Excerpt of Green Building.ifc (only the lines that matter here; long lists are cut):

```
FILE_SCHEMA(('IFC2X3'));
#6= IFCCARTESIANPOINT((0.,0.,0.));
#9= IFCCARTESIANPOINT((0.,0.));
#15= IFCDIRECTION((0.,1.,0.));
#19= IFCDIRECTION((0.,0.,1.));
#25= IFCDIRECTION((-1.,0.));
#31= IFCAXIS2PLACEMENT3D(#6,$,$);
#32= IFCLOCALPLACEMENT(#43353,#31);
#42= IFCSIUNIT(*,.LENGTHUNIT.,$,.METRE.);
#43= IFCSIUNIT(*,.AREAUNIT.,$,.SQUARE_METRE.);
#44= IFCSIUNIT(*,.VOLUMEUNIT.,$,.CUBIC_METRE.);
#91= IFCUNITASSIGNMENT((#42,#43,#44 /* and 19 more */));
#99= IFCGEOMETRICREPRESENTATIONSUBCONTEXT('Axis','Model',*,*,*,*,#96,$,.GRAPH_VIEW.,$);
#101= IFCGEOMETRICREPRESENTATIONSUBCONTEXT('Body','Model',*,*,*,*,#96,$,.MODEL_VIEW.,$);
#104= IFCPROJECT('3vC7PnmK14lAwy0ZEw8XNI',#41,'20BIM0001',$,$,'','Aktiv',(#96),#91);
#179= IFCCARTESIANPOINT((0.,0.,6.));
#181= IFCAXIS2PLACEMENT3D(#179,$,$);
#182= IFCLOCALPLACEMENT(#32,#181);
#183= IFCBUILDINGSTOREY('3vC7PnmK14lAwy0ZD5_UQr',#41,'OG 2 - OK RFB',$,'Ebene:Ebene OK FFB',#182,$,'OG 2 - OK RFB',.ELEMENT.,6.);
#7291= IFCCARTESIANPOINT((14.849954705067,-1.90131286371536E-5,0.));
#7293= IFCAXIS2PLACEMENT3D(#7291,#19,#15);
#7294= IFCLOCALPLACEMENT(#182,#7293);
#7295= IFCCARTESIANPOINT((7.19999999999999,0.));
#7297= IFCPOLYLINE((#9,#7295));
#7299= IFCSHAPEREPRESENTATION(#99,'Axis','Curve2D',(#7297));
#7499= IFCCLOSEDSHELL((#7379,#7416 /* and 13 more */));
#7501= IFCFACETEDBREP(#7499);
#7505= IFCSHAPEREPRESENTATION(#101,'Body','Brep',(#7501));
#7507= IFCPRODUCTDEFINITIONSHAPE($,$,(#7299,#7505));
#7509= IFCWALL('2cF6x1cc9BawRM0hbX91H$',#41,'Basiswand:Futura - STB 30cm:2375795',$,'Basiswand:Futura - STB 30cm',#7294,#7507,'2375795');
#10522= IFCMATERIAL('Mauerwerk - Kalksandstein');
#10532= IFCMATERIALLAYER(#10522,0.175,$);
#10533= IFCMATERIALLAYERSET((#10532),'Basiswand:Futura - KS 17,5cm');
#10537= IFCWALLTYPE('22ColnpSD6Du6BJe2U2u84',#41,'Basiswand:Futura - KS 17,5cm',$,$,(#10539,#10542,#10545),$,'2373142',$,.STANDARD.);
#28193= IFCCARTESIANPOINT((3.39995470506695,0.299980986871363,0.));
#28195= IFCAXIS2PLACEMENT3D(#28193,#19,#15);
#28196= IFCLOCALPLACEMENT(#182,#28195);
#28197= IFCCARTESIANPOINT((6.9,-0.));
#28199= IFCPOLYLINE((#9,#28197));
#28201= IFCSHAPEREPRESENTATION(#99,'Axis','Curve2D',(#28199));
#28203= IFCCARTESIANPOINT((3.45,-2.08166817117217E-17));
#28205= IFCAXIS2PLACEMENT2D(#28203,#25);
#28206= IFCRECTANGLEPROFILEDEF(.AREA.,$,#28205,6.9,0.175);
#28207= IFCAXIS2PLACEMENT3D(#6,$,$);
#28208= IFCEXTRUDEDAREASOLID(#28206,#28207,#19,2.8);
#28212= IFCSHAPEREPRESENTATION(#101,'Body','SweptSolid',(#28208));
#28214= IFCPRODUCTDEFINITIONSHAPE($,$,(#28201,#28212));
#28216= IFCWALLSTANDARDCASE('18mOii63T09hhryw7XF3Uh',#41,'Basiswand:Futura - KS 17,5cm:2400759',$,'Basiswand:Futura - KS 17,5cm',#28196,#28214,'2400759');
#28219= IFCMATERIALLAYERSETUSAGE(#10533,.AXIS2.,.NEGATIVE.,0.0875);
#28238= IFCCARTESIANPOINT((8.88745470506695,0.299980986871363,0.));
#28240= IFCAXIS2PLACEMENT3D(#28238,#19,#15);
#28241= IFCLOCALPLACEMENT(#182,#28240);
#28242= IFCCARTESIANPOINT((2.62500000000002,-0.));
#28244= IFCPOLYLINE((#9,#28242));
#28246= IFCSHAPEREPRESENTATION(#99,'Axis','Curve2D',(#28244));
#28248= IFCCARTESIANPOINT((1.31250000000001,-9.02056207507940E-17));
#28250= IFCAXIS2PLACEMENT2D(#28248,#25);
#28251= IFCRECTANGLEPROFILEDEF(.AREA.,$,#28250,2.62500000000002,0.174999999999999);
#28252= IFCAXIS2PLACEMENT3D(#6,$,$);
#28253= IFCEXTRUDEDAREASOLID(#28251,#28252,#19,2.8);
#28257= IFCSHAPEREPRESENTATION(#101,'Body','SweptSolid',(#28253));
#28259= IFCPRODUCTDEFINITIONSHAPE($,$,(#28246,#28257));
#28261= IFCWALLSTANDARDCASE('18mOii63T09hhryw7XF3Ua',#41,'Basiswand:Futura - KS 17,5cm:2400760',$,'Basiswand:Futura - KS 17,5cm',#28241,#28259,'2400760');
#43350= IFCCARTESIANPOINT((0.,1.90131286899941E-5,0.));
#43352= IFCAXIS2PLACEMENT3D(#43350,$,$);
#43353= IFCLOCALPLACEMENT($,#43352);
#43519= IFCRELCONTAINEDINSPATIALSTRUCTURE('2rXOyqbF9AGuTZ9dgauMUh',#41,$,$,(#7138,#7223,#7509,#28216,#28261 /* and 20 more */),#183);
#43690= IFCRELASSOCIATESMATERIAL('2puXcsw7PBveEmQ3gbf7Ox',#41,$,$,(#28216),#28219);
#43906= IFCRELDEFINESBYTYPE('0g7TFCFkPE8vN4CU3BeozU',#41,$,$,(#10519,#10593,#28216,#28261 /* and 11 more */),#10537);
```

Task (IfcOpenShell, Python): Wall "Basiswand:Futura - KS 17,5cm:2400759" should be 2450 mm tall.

```python
import ifcopenshell
import ifcopenshell.geom
import ifcopenshell.util.representation
import ifcopenshell.util.shape
import ifcopenshell.util.unit

model = ifcopenshell.open("Green Building.ifc")
unit_scale = ifcopenshell.util.unit.calculate_unit_scale(model)
settings = ifcopenshell.geom.settings()


def volume(element):
    """Net volume in cubic metres, openings subtracted."""
    shape = ifcopenshell.geom.create_shape(settings, element)
    return ifcopenshell.util.shape.get_volume(shape.geometry)


wall = model.by_id(28216)
before = volume(wall)

body = ifcopenshell.util.representation.get_representation(wall, "Model", "Body")
solid = body.Items[0]
old_height = solid.Depth
solid.Depth = 2.45 / unit_scale
after = volume(wall)

print(f"height {old_height:g} -> {solid.Depth:g}, volume {before:.3f} -> {after:.3f} m3")

model.write("Green Building-out.ifc")
```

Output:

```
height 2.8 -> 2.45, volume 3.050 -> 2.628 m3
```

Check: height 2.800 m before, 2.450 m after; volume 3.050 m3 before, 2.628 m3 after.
